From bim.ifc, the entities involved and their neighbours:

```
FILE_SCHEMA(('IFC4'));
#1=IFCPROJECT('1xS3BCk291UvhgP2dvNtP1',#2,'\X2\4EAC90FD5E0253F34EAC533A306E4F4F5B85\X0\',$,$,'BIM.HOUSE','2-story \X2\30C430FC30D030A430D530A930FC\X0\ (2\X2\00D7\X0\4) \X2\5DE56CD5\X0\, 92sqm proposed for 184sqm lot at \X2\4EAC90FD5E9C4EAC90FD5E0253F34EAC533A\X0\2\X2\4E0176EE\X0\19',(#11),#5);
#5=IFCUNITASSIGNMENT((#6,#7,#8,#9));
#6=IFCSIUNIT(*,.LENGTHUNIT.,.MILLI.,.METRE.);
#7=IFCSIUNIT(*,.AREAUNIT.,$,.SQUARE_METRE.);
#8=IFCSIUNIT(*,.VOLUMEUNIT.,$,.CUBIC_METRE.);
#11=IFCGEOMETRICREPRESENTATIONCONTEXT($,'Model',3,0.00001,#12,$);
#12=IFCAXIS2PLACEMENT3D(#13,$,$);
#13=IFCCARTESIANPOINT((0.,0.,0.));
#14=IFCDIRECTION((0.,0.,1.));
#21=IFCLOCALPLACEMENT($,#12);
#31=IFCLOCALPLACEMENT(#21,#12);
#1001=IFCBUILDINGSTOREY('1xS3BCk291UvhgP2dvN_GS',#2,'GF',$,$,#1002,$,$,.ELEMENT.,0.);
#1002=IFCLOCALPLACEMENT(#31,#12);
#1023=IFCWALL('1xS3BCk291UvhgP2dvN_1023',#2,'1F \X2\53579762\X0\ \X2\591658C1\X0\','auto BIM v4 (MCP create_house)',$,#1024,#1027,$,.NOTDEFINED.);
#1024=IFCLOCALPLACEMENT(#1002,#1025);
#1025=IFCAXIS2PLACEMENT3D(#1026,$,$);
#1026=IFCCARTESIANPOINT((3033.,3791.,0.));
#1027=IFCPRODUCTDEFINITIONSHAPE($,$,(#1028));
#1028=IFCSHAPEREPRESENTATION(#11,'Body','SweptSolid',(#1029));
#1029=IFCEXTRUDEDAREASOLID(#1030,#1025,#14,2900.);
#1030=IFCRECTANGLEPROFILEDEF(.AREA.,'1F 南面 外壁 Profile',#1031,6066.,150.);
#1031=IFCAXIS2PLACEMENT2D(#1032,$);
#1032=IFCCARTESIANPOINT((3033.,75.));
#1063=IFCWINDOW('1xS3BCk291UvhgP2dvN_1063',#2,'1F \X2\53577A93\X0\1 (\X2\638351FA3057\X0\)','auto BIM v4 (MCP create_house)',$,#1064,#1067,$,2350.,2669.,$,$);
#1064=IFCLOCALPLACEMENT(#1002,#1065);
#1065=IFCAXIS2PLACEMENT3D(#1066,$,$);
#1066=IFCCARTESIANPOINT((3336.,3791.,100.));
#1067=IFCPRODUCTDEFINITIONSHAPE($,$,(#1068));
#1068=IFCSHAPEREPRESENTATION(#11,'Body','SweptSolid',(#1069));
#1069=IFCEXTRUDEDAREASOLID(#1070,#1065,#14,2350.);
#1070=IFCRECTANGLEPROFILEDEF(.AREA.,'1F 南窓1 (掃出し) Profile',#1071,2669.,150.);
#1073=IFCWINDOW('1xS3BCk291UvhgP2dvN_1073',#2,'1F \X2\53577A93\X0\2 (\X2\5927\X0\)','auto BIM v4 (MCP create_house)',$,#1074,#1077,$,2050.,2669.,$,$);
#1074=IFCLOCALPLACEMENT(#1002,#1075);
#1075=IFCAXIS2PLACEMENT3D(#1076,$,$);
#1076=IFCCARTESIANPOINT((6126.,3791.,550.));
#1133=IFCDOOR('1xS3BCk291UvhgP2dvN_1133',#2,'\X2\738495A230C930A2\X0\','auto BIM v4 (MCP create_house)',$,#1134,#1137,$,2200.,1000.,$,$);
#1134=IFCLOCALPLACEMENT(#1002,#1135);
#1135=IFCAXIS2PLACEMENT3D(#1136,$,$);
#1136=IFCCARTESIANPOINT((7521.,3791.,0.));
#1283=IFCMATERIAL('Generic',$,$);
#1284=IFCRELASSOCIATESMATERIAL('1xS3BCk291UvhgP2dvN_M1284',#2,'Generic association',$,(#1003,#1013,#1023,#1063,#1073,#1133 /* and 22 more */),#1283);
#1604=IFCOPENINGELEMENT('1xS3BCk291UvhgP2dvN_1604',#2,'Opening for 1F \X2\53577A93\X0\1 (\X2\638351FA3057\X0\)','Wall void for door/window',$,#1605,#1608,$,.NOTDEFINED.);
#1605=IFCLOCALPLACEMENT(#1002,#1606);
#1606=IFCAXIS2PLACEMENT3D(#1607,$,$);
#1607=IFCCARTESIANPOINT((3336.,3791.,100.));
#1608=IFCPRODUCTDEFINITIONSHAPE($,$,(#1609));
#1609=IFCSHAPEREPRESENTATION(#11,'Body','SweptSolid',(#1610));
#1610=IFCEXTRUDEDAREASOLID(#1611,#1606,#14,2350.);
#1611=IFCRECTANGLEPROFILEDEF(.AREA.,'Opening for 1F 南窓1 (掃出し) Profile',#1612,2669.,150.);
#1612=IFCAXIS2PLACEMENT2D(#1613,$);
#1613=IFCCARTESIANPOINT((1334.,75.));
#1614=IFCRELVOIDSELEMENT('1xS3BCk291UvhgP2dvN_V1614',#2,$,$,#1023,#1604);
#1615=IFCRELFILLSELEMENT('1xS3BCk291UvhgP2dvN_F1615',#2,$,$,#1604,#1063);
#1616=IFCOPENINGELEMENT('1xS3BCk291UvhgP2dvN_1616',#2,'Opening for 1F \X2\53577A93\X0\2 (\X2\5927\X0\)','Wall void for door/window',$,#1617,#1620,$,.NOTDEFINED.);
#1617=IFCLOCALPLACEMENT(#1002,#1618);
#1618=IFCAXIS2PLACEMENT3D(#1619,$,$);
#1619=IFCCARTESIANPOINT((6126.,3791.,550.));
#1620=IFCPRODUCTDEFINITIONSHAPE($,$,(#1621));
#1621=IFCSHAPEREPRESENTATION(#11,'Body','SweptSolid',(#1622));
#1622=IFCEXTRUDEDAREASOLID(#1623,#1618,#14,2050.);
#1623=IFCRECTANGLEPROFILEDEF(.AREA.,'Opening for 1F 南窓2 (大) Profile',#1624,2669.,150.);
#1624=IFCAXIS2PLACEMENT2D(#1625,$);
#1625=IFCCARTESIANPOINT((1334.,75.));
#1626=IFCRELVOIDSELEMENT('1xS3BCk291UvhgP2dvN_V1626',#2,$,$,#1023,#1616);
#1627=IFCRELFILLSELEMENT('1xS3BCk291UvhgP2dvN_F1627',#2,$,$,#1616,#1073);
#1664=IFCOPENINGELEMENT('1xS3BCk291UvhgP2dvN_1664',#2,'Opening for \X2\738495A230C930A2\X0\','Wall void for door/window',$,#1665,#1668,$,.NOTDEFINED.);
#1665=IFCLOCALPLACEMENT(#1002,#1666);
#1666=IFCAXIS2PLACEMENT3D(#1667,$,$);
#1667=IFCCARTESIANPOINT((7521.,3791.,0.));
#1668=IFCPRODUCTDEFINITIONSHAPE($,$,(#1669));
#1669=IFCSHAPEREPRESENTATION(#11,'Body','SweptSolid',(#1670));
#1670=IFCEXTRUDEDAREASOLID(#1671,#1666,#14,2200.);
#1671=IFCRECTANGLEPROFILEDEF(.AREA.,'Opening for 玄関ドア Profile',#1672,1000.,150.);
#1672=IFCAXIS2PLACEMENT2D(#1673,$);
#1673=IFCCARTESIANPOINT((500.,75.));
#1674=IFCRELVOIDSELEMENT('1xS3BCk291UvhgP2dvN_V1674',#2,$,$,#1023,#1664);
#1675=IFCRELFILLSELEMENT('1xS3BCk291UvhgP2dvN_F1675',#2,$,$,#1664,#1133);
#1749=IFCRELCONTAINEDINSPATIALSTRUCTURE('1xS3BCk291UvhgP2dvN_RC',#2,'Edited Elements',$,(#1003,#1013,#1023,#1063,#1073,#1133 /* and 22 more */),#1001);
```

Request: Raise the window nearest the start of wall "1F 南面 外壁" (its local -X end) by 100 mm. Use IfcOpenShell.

```python
import numpy as np
import ifcopenshell
import ifcopenshell.api.geometry
import ifcopenshell.util.placement
import ifcopenshell.util.unit

model = ifcopenshell.open("bim.ifc")
unit_scale = ifcopenshell.util.unit.calculate_unit_scale(model)

window = model.by_guid("1xS3BCk291UvhgP2dvN_1063")
opening = window.FillsVoids[0].RelatingOpeningElement
dz = 0.1 / unit_scale

shift = np.array([0.0, 0.0, dz])
# The window is not placed relative to its opening, so move both.
for product in (opening, window):
    matrix = ifcopenshell.util.placement.get_local_placement(product.ObjectPlacement)
    matrix[:3, 3] += shift
    ifcopenshell.api.geometry.edit_object_placement(model, product=product, matrix=matrix, is_si=False)

print(f"moved by {dz * unit_scale:+.3f} m")

model.write("bim_edited.ifc")
```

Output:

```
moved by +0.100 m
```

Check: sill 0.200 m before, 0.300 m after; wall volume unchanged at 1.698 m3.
